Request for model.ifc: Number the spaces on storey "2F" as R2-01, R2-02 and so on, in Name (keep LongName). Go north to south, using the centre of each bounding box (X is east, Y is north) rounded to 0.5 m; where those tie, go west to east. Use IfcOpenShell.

First a look at what the model holds.

```python
import ifcopenshell
import ifcopenshell.util.element
import ifcopenshell.util.placement

model = ifcopenshell.open("model.ifc")
print(model.schema)
storey = next(s for s in model.by_type("IfcBuildingStorey") if s.Name == "2F")
spaces = [e for e in ifcopenshell.util.element.get_decomposition(storey) if e.is_a("IfcSpace")]
for e in sorted(spaces, key=lambda e: e.id()):
    origin = ifcopenshell.util.placement.get_local_placement(e.ObjectPlacement)[:3, 3]
    print(e.id(), e.Name, e.LongName, origin.round(2) + 0.0, sep=" | ")
```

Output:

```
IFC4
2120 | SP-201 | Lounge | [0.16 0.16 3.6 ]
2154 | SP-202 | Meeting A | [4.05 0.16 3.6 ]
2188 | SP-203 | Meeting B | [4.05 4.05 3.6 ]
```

```python
import ifcopenshell
import ifcopenshell.geom
import ifcopenshell.util.element
import ifcopenshell.util.shape

model = ifcopenshell.open("model.ifc")
settings = ifcopenshell.geom.settings()
settings.set("use-world-coords", True)


def centre(element):
    shape = ifcopenshell.geom.create_shape(settings, element)
    return ifcopenshell.util.shape.get_bbox_centroid(shape.geometry)


storey = next(s for s in model.by_type("IfcBuildingStorey") if s.Name == "2F")
spaces = [e for e in ifcopenshell.util.element.get_decomposition(storey) if e.is_a("IfcSpace")]

# Insertion points can sit at a corner or the storey origin, so sort by the geometry (in metres).
centres = {e: centre(e) for e in spaces}
spaces.sort(key=lambda e: (-round(centres[e][1] / 0.5), centres[e][0]))

for i, e in enumerate(spaces, start=1):
    number = f"R2-{i:02d}"
    e.Name = number
    print(e.id(), number)

model.write("model-out.ifc")
```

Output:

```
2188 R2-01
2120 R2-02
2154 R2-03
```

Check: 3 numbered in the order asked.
